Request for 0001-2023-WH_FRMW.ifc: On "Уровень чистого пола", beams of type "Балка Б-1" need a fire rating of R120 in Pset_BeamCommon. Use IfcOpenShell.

First a look at what the model holds.

```python
import ifcopenshell
import ifcopenshell.util.element

model = ifcopenshell.open("0001-2023-WH_FRMW.ifc")
print(model.schema)
storey = next(s for s in model.by_type("IfcBuildingStorey") if s.Name == "Уровень чистого пола")
beams = [e for e in ifcopenshell.util.element.get_decomposition(storey) if e.is_a("IfcBeam")]
seen = {}
for e in beams:
    element_type = ifcopenshell.util.element.get_type(e)
    key = (element_type.Name if element_type != e and element_type else None, ifcopenshell.util.element.get_pset(e, "Pset_BeamCommon", "FireRating"))
    seen[key] = seen.get(key, 0) + 1
for (name, value), count in sorted(seen.items(), key=str):
    print(count, "x", name, "|", value)
```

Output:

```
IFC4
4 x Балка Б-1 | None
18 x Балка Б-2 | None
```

```python
import ifcopenshell
import ifcopenshell.api.pset
import ifcopenshell.util.element

model = ifcopenshell.open("0001-2023-WH_FRMW.ifc")

storey = next(s for s in model.by_type("IfcBuildingStorey") if s.Name == "Уровень чистого пола")
beams = [e for e in ifcopenshell.util.element.get_decomposition(storey) if e.is_a("IfcBeam")]

count = 0
for e in beams:
    element_type = ifcopenshell.util.element.get_type(e)
    if element_type in (None, e) or element_type.Name != "Балка Б-1":
        continue
    # add_pset returns the element's existing set when there is one.
    pset = ifcopenshell.api.pset.add_pset(model, product=e, name="Pset_BeamCommon")
    ifcopenshell.api.pset.edit_pset(model, pset=pset, properties={"FireRating": "R120"})
    count += 1

print(count, "beams updated")

model.write("0001-2023-WH_FRMW_rev.ifc")
```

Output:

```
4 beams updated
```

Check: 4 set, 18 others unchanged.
